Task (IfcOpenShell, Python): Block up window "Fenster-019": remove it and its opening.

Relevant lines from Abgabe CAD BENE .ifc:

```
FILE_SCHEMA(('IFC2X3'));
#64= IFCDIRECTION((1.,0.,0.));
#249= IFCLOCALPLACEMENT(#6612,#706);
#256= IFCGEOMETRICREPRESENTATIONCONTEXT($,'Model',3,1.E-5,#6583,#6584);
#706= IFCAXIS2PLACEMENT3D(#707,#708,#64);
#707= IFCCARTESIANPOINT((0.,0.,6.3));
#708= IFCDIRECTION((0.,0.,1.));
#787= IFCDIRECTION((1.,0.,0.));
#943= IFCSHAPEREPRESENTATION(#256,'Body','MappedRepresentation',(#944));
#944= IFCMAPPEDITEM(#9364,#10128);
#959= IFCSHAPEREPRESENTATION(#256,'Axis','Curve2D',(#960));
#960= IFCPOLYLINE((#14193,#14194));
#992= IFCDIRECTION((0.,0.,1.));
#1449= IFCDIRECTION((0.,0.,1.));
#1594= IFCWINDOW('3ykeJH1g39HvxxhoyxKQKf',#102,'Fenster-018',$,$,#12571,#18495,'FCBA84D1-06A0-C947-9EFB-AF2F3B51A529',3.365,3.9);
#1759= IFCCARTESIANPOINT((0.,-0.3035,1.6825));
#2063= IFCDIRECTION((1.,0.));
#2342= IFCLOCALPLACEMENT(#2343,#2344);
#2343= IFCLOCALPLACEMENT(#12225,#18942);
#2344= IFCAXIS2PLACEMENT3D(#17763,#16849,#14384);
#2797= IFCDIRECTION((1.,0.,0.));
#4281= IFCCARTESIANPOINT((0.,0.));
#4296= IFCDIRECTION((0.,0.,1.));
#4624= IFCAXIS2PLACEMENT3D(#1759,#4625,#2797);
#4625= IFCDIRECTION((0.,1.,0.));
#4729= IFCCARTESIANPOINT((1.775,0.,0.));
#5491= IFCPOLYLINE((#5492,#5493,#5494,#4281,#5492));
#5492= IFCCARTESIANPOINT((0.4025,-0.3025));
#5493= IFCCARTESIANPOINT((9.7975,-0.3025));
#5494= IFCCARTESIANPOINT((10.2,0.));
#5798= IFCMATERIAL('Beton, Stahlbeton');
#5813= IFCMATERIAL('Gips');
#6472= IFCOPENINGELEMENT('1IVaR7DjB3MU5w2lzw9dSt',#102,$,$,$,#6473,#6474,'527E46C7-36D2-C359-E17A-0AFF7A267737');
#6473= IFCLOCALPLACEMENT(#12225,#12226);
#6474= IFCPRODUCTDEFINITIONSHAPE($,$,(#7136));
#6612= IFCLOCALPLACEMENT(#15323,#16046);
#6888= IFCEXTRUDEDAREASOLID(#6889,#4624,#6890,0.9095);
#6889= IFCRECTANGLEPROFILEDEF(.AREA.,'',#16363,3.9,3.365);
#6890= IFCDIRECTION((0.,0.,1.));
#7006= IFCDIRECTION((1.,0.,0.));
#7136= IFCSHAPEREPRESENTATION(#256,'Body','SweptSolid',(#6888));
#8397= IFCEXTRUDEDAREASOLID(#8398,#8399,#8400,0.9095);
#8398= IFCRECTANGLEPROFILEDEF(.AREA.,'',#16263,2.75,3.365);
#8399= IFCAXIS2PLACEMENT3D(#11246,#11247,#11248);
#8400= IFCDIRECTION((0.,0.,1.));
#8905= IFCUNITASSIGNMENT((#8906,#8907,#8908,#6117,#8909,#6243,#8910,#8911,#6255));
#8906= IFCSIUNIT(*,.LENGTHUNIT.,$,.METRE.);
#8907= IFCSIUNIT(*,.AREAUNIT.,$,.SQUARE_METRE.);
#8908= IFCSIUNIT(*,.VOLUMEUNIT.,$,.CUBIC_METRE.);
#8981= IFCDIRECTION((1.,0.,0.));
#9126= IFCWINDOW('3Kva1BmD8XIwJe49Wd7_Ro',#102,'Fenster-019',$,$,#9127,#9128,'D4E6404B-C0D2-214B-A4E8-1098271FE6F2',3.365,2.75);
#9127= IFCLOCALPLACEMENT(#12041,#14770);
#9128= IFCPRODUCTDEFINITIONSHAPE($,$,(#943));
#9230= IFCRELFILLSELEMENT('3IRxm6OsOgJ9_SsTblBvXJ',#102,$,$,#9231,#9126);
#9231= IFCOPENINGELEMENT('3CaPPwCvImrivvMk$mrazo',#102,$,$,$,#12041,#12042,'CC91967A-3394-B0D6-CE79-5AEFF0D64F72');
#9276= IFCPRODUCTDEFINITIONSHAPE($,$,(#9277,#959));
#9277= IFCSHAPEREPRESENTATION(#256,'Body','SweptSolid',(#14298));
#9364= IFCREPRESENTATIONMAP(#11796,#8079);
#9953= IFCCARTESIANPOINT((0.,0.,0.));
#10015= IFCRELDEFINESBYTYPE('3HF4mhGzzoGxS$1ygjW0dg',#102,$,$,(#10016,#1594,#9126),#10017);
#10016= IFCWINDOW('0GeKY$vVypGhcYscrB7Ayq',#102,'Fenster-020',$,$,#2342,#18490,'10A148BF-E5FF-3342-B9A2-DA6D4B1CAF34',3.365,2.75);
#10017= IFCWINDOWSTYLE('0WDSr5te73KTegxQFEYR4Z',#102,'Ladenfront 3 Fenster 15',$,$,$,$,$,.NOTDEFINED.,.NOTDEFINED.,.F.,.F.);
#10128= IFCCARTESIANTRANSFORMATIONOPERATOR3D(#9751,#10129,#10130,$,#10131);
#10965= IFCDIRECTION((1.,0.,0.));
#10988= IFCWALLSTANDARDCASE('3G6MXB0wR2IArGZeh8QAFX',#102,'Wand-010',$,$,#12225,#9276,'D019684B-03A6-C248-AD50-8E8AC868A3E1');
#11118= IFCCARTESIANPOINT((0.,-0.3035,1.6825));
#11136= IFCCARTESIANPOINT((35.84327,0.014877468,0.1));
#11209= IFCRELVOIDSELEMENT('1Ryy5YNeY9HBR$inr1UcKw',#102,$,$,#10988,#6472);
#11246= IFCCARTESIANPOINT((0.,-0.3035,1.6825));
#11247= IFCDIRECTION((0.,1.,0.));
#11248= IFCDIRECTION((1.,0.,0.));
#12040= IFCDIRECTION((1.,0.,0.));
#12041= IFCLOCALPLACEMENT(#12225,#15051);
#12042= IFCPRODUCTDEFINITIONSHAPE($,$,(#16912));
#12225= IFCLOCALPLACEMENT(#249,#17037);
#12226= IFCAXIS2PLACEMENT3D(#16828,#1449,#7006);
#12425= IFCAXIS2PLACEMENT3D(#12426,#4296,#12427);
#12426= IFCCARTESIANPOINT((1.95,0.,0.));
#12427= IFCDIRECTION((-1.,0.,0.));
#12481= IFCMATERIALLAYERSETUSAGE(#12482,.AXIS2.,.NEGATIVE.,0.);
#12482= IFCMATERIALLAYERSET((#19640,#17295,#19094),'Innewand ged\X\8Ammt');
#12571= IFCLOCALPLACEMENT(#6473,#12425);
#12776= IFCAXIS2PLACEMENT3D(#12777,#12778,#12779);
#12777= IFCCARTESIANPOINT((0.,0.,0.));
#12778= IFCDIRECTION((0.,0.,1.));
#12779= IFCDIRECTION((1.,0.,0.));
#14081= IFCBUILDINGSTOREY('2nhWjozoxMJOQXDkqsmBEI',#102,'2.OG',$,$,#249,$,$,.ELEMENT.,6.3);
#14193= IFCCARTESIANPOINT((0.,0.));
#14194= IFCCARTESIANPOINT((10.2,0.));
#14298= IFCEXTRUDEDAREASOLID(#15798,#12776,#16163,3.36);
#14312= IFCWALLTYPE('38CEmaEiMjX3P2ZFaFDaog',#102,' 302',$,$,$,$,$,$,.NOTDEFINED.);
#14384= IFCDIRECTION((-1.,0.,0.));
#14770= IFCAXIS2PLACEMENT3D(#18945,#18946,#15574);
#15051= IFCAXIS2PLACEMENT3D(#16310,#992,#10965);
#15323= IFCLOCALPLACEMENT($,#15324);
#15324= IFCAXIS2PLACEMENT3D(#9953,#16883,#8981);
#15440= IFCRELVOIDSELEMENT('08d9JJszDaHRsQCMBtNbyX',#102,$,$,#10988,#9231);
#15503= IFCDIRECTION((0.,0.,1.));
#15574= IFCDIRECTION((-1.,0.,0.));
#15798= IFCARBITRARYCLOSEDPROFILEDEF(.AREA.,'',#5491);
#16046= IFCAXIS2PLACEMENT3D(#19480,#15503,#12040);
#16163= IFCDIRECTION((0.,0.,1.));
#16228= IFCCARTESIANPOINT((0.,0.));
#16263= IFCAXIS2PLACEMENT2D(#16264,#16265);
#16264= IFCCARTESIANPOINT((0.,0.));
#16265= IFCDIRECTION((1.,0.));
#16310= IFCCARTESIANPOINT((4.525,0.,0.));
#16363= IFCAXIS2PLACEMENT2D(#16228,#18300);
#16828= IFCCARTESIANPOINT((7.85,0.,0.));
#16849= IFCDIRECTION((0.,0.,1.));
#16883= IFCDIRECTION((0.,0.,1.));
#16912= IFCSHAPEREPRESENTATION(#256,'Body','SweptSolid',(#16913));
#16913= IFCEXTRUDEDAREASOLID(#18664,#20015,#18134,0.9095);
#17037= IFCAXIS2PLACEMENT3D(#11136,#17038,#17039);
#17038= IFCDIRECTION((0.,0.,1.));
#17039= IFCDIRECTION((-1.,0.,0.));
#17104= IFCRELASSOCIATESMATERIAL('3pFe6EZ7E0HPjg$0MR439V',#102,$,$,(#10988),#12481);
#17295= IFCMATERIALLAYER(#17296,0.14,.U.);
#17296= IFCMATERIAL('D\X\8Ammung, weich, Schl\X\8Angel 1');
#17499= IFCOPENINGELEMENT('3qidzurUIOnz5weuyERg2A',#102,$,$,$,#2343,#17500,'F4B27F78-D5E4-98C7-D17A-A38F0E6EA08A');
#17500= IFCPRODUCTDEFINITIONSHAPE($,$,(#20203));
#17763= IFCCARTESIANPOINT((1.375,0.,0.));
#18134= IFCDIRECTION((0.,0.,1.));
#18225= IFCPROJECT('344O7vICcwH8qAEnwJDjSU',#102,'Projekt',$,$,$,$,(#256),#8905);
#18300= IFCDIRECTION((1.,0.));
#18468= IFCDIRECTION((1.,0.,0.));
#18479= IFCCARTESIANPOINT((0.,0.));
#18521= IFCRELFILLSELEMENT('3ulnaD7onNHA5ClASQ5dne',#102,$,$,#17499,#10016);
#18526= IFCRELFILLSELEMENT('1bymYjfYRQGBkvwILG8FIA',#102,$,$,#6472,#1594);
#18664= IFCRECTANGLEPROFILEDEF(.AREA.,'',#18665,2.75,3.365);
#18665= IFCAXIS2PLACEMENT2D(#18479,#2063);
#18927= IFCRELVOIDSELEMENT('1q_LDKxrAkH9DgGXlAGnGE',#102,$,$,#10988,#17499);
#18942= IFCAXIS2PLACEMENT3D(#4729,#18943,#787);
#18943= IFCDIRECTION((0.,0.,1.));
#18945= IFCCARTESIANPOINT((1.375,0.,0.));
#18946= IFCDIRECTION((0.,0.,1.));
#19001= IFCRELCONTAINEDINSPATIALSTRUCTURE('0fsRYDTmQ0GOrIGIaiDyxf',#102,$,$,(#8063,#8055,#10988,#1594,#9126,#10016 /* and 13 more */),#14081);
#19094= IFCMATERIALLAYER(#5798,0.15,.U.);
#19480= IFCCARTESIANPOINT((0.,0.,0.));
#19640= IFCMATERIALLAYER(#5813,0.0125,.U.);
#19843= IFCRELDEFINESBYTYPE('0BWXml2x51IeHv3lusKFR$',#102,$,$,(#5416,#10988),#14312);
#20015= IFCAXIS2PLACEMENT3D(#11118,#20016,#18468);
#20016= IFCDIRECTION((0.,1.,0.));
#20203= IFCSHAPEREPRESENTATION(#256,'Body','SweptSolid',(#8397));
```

```python
import ifcopenshell
import ifcopenshell.api.feature
import ifcopenshell.api.root
import ifcopenshell.geom
import ifcopenshell.util.shape

model = ifcopenshell.open("Abgabe CAD BENE .ifc")
settings = ifcopenshell.geom.settings()


def volume(element):
    """Net volume in cubic metres, openings subtracted."""
    shape = ifcopenshell.geom.create_shape(settings, element)
    return ifcopenshell.util.shape.get_volume(shape.geometry)


window = model.by_guid("3Kva1BmD8XIwJe49Wd7_Ro")
opening = window.FillsVoids[0].RelatingOpeningElement
wall = opening.VoidsElements[0].RelatingBuildingElement
before = volume(wall)

ifcopenshell.api.root.remove_product(model, product=window)
ifcopenshell.api.feature.remove_feature(model, feature=opening)

after = volume(wall)

print(f"wall volume {before:.3f} -> {after:.3f} m3")

model.write("Abgabe CAD BENE _updated.ifc")
```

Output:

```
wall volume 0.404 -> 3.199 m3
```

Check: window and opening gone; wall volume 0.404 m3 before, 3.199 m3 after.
